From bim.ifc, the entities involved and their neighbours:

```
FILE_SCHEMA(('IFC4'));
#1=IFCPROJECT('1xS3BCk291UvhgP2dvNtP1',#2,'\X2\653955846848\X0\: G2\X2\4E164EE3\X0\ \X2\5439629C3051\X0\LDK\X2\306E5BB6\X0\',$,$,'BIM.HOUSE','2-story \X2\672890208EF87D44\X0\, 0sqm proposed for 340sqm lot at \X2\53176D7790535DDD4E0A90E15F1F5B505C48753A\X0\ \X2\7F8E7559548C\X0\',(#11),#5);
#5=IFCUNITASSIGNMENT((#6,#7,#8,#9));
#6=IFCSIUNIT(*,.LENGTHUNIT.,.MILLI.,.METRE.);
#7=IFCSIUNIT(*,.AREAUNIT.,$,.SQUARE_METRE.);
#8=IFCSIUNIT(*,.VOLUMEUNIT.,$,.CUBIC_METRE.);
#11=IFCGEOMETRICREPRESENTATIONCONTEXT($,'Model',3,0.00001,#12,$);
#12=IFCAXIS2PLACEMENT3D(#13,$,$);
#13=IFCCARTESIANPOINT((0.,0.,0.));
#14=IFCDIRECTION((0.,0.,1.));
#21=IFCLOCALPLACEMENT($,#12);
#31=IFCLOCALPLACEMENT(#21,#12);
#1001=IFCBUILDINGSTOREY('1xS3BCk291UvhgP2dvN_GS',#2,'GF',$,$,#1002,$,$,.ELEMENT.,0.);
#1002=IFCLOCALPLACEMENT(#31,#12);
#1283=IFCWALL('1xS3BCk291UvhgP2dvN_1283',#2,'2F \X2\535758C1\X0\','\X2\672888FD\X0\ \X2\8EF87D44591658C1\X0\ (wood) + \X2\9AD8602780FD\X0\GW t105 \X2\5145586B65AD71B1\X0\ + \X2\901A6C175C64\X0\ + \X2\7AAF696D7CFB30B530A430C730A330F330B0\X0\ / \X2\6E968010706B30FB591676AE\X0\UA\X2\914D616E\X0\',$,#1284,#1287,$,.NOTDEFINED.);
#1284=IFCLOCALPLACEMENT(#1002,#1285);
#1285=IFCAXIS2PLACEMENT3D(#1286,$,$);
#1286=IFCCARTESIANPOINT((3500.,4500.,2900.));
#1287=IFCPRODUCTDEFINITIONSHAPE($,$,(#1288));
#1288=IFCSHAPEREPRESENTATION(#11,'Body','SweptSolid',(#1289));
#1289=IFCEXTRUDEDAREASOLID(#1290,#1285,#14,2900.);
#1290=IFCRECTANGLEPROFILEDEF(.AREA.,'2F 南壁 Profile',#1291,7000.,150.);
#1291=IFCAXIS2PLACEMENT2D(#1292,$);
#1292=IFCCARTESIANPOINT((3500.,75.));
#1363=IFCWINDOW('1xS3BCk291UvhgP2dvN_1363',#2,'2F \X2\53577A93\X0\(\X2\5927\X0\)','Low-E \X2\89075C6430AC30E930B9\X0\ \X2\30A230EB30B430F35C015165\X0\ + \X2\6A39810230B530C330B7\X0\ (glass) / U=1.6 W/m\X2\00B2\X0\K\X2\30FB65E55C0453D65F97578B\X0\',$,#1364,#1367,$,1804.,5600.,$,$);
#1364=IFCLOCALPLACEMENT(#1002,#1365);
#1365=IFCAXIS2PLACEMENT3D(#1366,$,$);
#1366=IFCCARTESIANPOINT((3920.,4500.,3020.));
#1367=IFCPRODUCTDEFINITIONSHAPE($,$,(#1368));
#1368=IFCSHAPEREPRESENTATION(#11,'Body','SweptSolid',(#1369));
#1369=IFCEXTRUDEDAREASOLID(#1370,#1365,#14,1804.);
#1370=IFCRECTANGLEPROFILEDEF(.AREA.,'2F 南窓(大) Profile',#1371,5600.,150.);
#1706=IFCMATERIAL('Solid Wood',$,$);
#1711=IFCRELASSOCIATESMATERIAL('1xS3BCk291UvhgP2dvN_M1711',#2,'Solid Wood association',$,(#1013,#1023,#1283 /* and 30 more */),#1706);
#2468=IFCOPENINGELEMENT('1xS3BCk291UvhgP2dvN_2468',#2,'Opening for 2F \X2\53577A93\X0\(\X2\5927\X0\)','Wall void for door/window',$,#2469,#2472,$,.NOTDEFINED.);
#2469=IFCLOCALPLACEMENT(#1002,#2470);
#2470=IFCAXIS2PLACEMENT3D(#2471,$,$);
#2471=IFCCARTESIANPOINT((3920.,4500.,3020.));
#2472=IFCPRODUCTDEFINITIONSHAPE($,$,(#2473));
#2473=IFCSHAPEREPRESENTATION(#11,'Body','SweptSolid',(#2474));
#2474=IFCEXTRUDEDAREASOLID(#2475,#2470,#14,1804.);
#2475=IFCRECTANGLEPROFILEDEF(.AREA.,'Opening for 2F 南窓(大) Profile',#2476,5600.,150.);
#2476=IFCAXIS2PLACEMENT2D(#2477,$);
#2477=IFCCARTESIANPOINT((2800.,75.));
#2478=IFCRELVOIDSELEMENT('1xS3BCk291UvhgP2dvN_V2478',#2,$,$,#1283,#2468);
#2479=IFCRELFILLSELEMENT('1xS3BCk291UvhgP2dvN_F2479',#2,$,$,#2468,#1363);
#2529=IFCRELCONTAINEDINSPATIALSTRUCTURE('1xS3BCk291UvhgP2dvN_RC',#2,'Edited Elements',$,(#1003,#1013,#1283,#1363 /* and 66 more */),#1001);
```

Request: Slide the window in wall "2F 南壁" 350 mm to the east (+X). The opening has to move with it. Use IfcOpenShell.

```python
import ifcopenshell
import ifcopenshell.api.geometry
import ifcopenshell.util.placement
import ifcopenshell.util.unit

model = ifcopenshell.open("bim.ifc")
unit_scale = ifcopenshell.util.unit.calculate_unit_scale(model)

window = model.by_id(1363)
opening = window.FillsVoids[0].RelatingOpeningElement
wall = opening.VoidsElements[0].RelatingBuildingElement

wall_matrix = ifcopenshell.util.placement.get_local_placement(wall.ObjectPlacement)
shift = wall_matrix[:3, 0] * 0.35 / unit_scale
before = ifcopenshell.util.placement.get_local_placement(window.ObjectPlacement)[:3, 3].copy()

# The window is not placed relative to its opening, so move both.
for product in (opening, window):
    matrix = ifcopenshell.util.placement.get_local_placement(product.ObjectPlacement)
    matrix[:3, 3] += shift
    ifcopenshell.api.geometry.edit_object_placement(model, product=product, matrix=matrix, is_si=False)

after = ifcopenshell.util.placement.get_local_placement(window.ObjectPlacement)[:3, 3]
print("window moved by", (after - before).round(3) + 0.0)

model.write("bim_rev.ifc")
```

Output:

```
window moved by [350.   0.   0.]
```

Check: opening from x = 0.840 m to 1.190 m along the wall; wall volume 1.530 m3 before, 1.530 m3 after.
